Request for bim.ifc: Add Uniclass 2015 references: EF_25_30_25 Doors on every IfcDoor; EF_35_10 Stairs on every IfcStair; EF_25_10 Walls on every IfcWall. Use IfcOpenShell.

First a look at what the model holds.

```python
import ifcopenshell

model = ifcopenshell.open("bim.ifc")
print(model.schema)
print("classifications:", [c.Name for c in model.by_type("IfcClassification")])
for ifc_class in ("IfcDoor", "IfcRoof", "IfcStair", "IfcWall", "IfcWindow"):
    print(ifc_class, len(model.by_type(ifc_class)))
```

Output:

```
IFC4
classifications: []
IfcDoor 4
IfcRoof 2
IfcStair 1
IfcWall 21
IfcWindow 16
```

```python
import ifcopenshell
import ifcopenshell.api.classification

model = ifcopenshell.open("bim.ifc")

system = ifcopenshell.api.classification.add_classification(model, classification="Uniclass 2015")

codes = {
    "IfcDoor": ("EF_25_30_25", "Doors"),
    "IfcStair": ("EF_35_10", "Stairs"),
    "IfcWall": ("EF_25_10", "Walls"),
}
for ifc_class, (code, name) in codes.items():
    products = model.by_type(ifc_class)
    ifcopenshell.api.classification.add_reference(
        model, products=products, classification=system, identification=code, name=name
    )
    print(code, len(products))

model.write("bim-out.ifc")
```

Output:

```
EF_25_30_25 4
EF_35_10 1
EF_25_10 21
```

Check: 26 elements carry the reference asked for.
